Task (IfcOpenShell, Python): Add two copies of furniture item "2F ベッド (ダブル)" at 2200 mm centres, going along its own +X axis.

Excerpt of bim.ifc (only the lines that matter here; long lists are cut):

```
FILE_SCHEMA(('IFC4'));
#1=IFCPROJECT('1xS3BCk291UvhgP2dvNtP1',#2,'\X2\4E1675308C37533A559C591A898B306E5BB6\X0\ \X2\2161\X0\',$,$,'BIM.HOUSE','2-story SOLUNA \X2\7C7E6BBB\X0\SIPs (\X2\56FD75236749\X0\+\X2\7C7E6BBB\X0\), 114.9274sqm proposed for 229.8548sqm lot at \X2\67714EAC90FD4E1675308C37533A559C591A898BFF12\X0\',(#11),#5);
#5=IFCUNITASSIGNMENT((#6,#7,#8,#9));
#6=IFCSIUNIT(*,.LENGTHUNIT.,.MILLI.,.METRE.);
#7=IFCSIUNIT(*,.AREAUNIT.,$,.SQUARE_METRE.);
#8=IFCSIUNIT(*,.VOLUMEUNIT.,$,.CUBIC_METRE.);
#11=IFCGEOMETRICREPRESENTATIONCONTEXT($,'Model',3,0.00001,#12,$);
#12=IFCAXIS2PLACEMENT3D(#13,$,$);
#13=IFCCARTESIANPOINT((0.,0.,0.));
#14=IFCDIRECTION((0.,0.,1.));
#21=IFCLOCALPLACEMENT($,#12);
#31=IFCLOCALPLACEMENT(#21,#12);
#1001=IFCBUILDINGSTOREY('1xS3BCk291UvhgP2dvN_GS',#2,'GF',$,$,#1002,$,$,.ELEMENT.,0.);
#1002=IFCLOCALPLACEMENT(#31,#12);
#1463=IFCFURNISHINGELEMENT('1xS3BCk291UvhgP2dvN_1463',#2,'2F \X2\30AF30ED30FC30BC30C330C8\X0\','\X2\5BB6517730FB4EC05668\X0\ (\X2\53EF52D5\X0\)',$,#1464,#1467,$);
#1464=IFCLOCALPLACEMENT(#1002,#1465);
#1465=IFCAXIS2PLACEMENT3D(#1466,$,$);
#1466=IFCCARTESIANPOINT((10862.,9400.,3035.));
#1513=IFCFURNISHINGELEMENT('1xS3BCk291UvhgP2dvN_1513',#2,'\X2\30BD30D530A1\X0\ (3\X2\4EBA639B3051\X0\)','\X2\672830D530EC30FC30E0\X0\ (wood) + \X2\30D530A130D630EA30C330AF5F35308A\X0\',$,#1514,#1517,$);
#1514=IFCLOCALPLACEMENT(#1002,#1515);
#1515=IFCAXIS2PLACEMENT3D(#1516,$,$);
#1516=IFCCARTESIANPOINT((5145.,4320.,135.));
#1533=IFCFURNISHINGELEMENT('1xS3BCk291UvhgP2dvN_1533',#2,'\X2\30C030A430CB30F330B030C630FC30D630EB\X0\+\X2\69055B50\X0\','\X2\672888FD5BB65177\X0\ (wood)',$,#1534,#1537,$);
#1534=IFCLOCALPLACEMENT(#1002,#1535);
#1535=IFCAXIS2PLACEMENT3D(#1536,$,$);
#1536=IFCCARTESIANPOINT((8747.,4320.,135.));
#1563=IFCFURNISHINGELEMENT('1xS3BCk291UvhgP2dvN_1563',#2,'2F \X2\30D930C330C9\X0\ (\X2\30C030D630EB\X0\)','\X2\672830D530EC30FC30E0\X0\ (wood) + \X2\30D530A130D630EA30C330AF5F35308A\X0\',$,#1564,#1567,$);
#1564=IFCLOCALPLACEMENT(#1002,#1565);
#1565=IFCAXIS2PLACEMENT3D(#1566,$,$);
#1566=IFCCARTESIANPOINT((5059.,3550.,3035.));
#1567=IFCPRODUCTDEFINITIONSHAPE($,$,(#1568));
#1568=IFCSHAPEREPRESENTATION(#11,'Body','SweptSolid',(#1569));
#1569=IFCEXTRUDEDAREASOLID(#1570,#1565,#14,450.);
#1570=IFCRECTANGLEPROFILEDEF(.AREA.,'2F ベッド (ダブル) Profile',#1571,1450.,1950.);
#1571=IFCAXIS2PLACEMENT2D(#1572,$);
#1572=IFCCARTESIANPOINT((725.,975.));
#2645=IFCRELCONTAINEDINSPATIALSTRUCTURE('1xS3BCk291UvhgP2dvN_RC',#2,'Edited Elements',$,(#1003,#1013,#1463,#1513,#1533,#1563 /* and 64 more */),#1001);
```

```python
import ifcopenshell
import ifcopenshell.api.geometry
import ifcopenshell.api.root
import ifcopenshell.util.element
import ifcopenshell.util.placement
import ifcopenshell.util.unit

model = ifcopenshell.open("bim.ifc")
unit_scale = ifcopenshell.util.unit.calculate_unit_scale(model)


def reuse_history(source, copy):
    """copy_class also copies each property set's owner history, people and application; keep the originals."""
    for rel in copy.IsDefinedBy:
        if rel.is_a("IfcRelDefinesByProperties") and (history := rel.RelatingPropertyDefinition.OwnerHistory):
            rel.RelatingPropertyDefinition.OwnerHistory = source.OwnerHistory
            ifcopenshell.util.element.remove_deep2(model, history)


source = model.by_guid("1xS3BCk291UvhgP2dvN_1563")
base = ifcopenshell.util.placement.get_local_placement(source.ObjectPlacement)
step = base[:3, 0] * 2.2 / unit_scale

for i in range(1, 3):
    copy = ifcopenshell.api.root.copy_class(model, product=source)
    copy.Representation = ifcopenshell.util.element.copy_deep(
        model, source.Representation, exclude=["IfcGeometricRepresentationContext", "IfcRepresentationMap"]
    )
    reuse_history(source, copy)
    matrix = base.copy()
    matrix[:3, 3] += i * step
    print("added at", matrix[:3, 3].round(3) + 0.0)
    ifcopenshell.api.geometry.edit_object_placement(model, product=copy, matrix=matrix, is_si=False)

model.write("bim_v2.ifc")
```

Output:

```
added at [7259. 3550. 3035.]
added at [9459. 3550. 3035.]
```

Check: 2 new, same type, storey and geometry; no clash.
